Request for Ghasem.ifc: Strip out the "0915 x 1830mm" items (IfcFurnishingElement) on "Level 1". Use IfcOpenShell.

First a look at what the model holds.

```python
import ifcopenshell
import ifcopenshell.util.element

model = ifcopenshell.open("Ghasem.ifc")
print(model.schema)
storey = next(s for s in model.by_type("IfcBuildingStorey") if s.Name == "Level 1")
furniture = [e for e in ifcopenshell.util.element.get_decomposition(storey) if e.is_a("IfcFurnishingElement")]
seen = {}
for e in furniture:
    element_type = ifcopenshell.util.element.get_type(e)
    name = element_type.Name if element_type not in (None, e) else None
    seen[name] = seen.get(name, 0) + 1
for name, count in sorted(seen.items(), key=str):
    print(count, "x", name)
```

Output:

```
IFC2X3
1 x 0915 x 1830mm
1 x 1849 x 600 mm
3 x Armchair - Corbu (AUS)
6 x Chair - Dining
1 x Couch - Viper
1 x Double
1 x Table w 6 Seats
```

```python
import ifcopenshell
import ifcopenshell.api.root
import ifcopenshell.util.element

model = ifcopenshell.open("Ghasem.ifc")

storey = next(s for s in model.by_type("IfcBuildingStorey") if s.Name == "Level 1")
furniture = [e for e in ifcopenshell.util.element.get_decomposition(storey) if e.is_a("IfcFurnishingElement")]
targets = [e for e in furniture if (t := ifcopenshell.util.element.get_type(e)) not in (None, e) and t.Name == "0915 x 1830mm"]

for e in targets:
    ifcopenshell.api.root.remove_product(model, product=e)
print(len(targets), "removed")

model.write("Ghasem_updated.ifc")
```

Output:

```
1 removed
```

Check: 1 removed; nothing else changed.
